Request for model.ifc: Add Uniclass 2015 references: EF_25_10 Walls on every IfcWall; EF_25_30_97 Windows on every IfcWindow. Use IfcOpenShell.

First a look at what the model holds.

```python
import ifcopenshell

model = ifcopenshell.open("model.ifc")
print(model.schema)
print("classifications:", [c.Name for c in model.by_type("IfcClassification")])
for ifc_class in ("IfcDoor", "IfcRoof", "IfcStair", "IfcWall", "IfcWindow"):
    print(ifc_class, len(model.by_type(ifc_class)))
```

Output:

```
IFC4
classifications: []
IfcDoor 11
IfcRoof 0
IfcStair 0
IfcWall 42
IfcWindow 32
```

```python
import ifcopenshell
import ifcopenshell.api.classification

model = ifcopenshell.open("model.ifc")

system = ifcopenshell.api.classification.add_classification(model, classification="Uniclass 2015")

codes = {
    "IfcWall": ("EF_25_10", "Walls"),
    "IfcWindow": ("EF_25_30_97", "Windows"),
}
for ifc_class, (code, name) in codes.items():
    products = model.by_type(ifc_class)
    ifcopenshell.api.classification.add_reference(
        model, products=products, classification=system, identification=code, name=name
    )
    print(code, len(products))

model.write("model-out.ifc")
```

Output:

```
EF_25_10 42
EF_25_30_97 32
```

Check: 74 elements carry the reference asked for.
